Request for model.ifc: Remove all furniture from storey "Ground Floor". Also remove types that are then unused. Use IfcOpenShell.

First a look at what the model holds.

```python
import ifcopenshell
import ifcopenshell.util.element

model = ifcopenshell.open("model.ifc")
print(model.schema)
storey = next(s for s in model.by_type("IfcBuildingStorey") if s.Name == "Ground Floor")
furniture = [e for e in ifcopenshell.util.element.get_decomposition(storey) if e.is_a("IfcFurnishingElement")]
seen = {}
for e in furniture:
    element_type = ifcopenshell.util.element.get_type(e)
    name = element_type.Name if element_type not in (None, e) else None
    seen[name] = seen.get(name, 0) + 1
for name, count in sorted(seen.items(), key=str):
    print(count, "x", name)
```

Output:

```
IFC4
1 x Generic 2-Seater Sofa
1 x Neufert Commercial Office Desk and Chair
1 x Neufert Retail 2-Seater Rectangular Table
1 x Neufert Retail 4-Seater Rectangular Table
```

```python
import ifcopenshell
import ifcopenshell.api.root
import ifcopenshell.util.element

model = ifcopenshell.open("model.ifc")

storey = next(s for s in model.by_type("IfcBuildingStorey") if s.Name == "Ground Floor")
furniture = [e for e in ifcopenshell.util.element.get_decomposition(storey) if e.is_a("IfcFurnishingElement")]
types = {ifcopenshell.util.element.get_type(e) for e in furniture} - {None, *furniture}

for e in furniture:
    ifcopenshell.api.root.remove_product(model, product=e)
print(len(furniture), "removed")

unused = [t for t in types if not ifcopenshell.util.element.get_types(t)]
for t in unused:
    ifcopenshell.api.root.remove_product(model, product=t)
print(len(unused), "unused types removed")

model.write("model_rev.ifc")
```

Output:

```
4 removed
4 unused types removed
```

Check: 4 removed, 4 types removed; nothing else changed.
